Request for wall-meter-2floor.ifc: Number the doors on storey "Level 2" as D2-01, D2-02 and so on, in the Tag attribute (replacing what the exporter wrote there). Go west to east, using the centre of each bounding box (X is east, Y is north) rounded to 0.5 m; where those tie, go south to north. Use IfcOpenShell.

First a look at what the model holds.

```python
import ifcopenshell
import ifcopenshell.util.element
import ifcopenshell.util.placement

model = ifcopenshell.open("wall-meter-2floor.ifc")
print(model.schema)
storey = next(s for s in model.by_type("IfcBuildingStorey") if s.Name == "Level 2")
doors = [e for e in ifcopenshell.util.element.get_decomposition(storey) if e.is_a("IfcDoor")]
for e in sorted(doors, key=lambda e: e.id()):
    origin = ifcopenshell.util.placement.get_local_placement(e.ObjectPlacement)[:3, 3]
    print(e.id(), e.Tag, e.Name, origin.round(2) + 0.0, sep=" | ")
```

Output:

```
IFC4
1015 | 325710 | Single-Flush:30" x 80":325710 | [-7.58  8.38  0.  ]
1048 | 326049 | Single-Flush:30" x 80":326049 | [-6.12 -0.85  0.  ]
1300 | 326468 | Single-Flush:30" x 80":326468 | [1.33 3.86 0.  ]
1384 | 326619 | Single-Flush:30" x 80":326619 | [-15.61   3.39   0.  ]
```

```python
import ifcopenshell
import ifcopenshell.geom
import ifcopenshell.util.element
import ifcopenshell.util.shape

model = ifcopenshell.open("wall-meter-2floor.ifc")
settings = ifcopenshell.geom.settings()
settings.set("use-world-coords", True)


def centre(element):
    shape = ifcopenshell.geom.create_shape(settings, element)
    return ifcopenshell.util.shape.get_bbox_centroid(shape.geometry)


storey = next(s for s in model.by_type("IfcBuildingStorey") if s.Name == "Level 2")
doors = [e for e in ifcopenshell.util.element.get_decomposition(storey) if e.is_a("IfcDoor")]

# Insertion points can sit at a corner or the storey origin, so sort by the geometry (in metres).
centres = {e: centre(e) for e in doors}
doors.sort(key=lambda e: (round(centres[e][0] / 0.5), centres[e][1]))

for i, e in enumerate(doors, start=1):
    number = f"D2-{i:02d}"
    e.Tag = number
    print(e.id(), number)

model.write("wall-meter-2floor-out.ifc")
```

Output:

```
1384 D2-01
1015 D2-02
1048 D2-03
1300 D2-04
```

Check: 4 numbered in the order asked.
